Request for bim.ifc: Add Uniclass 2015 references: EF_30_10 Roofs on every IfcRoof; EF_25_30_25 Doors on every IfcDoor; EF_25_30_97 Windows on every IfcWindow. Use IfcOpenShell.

First a look at what the model holds.

```python
import ifcopenshell

model = ifcopenshell.open("bim.ifc")
print(model.schema)
print("classifications:", [c.Name for c in model.by_type("IfcClassification")])
for ifc_class in ("IfcDoor", "IfcRoof", "IfcStair", "IfcWall", "IfcWindow"):
    print(ifc_class, len(model.by_type(ifc_class)))
```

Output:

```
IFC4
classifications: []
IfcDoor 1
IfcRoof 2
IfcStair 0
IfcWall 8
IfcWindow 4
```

```python
import ifcopenshell
import ifcopenshell.api.classification

model = ifcopenshell.open("bim.ifc")

system = ifcopenshell.api.classification.add_classification(model, classification="Uniclass 2015")

codes = {
    "IfcRoof": ("EF_30_10", "Roofs"),
    "IfcDoor": ("EF_25_30_25", "Doors"),
    "IfcWindow": ("EF_25_30_97", "Windows"),
}
for ifc_class, (code, name) in codes.items():
    products = model.by_type(ifc_class)
    ifcopenshell.api.classification.add_reference(
        model, products=products, classification=system, identification=code, name=name
    )
    print(code, len(products))

model.write("bim_v2.ifc")
```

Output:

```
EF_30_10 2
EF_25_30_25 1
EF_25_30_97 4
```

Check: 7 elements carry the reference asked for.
